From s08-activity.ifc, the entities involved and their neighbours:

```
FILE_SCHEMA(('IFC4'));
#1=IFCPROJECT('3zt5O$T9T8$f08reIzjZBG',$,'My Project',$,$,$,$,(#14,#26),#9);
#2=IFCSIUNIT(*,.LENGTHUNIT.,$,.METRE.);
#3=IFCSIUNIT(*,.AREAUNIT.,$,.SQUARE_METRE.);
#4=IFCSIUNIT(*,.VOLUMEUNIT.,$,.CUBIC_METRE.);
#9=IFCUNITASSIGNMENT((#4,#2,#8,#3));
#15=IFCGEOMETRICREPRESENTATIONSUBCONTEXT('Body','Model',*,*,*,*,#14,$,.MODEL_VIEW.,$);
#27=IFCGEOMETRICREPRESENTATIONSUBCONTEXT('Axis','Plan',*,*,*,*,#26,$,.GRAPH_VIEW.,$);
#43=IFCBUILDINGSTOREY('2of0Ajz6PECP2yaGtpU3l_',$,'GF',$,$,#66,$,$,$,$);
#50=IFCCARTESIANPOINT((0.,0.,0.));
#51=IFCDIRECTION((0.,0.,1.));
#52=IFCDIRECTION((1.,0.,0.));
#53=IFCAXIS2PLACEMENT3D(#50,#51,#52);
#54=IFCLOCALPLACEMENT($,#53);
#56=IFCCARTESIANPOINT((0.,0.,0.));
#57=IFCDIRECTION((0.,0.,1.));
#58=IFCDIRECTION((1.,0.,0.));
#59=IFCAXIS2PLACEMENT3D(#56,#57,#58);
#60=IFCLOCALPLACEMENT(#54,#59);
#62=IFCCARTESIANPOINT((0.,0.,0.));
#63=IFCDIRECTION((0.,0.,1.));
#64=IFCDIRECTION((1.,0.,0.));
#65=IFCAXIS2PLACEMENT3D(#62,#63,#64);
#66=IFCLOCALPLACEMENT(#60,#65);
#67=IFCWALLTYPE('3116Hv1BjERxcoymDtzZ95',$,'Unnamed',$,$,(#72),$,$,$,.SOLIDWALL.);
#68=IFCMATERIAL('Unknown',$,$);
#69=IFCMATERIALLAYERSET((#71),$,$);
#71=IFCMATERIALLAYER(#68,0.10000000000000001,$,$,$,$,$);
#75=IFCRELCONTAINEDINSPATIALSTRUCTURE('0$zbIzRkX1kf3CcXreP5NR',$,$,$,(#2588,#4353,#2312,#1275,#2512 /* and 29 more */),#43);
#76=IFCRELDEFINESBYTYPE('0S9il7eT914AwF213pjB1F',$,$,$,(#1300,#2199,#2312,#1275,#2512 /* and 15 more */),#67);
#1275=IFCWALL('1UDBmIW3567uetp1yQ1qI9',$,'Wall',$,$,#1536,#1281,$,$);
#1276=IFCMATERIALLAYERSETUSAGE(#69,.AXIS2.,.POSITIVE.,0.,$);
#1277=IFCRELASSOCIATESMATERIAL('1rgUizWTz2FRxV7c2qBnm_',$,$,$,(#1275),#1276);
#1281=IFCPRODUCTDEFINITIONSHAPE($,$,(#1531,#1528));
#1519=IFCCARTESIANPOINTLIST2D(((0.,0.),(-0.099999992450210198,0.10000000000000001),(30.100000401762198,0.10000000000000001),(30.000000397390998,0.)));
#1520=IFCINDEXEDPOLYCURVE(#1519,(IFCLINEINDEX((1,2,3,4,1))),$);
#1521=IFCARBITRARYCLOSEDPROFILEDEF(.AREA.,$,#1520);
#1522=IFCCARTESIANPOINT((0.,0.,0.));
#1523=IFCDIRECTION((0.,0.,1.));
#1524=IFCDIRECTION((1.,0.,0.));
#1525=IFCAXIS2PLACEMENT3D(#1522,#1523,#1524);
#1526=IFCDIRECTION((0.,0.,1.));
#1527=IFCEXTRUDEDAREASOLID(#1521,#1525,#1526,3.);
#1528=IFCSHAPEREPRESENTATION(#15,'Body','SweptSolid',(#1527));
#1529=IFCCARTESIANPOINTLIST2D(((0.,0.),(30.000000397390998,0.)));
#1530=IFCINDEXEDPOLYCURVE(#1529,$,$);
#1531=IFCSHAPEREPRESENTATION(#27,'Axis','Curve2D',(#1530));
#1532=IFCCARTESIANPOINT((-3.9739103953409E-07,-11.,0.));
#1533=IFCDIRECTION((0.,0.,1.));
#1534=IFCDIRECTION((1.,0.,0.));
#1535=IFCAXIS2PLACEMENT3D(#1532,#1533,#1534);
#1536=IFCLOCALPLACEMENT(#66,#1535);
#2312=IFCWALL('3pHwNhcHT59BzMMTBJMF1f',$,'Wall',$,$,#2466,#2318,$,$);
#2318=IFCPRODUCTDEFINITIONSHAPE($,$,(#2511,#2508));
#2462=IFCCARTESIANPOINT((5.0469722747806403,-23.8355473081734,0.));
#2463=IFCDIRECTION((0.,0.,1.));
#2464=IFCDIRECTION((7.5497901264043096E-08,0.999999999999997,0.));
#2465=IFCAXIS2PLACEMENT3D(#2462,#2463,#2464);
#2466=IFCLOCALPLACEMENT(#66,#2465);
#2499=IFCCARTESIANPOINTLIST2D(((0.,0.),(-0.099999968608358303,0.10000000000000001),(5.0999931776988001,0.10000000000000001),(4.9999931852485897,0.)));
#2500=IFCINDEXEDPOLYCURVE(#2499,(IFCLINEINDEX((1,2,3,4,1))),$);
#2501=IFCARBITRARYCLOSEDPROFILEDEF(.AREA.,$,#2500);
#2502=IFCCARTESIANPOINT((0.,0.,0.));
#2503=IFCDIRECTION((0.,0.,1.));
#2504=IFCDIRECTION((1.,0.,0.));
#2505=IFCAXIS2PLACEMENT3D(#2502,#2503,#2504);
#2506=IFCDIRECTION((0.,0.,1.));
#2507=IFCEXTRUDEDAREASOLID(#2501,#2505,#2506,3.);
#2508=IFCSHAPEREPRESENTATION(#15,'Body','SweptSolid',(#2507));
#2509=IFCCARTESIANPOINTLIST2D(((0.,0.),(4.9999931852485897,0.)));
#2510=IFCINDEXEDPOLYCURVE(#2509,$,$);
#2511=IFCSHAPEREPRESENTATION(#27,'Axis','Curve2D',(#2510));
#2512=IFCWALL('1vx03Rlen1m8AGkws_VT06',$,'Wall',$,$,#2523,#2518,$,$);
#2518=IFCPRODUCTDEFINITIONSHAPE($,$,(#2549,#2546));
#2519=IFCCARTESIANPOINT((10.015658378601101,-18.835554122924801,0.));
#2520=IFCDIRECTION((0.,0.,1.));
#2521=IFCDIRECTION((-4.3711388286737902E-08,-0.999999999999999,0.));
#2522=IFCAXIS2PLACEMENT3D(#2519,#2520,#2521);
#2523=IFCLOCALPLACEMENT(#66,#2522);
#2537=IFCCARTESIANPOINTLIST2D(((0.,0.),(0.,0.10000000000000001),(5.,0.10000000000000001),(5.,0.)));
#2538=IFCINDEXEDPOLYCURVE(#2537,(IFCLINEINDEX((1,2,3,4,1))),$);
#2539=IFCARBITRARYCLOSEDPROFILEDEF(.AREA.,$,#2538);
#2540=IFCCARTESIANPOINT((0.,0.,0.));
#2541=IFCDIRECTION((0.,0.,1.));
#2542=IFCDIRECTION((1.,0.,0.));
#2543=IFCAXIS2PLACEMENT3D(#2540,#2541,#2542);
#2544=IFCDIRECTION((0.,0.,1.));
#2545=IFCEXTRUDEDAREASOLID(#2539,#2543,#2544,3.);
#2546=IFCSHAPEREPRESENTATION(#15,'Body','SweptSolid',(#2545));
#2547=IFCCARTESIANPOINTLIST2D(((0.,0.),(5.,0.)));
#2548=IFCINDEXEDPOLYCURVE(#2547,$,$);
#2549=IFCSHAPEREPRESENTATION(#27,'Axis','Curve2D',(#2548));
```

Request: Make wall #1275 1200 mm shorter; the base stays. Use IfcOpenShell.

```python
import ifcopenshell
import ifcopenshell.geom
import ifcopenshell.util.representation
import ifcopenshell.util.shape
import ifcopenshell.util.unit

model = ifcopenshell.open("s08-activity.ifc")
unit_scale = ifcopenshell.util.unit.calculate_unit_scale(model)
settings = ifcopenshell.geom.settings()


def volume(element):
    """Net volume in cubic metres, openings subtracted."""
    shape = ifcopenshell.geom.create_shape(settings, element)
    return ifcopenshell.util.shape.get_volume(shape.geometry)


wall = model.by_guid("1UDBmIW3567uetp1yQ1qI9")
before = volume(wall)

body = ifcopenshell.util.representation.get_representation(wall, "Model", "Body")
solid = body.Items[0]
old_height = solid.Depth
solid.Depth -= 1.2 / unit_scale
after = volume(wall)

print(f"height {old_height:g} -> {solid.Depth:g}, volume {before:.3f} -> {after:.3f} m3")

model.write("s08-activity-out.ifc")
```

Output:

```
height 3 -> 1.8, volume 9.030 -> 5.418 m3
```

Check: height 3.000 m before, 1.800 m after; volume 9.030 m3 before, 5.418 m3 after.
